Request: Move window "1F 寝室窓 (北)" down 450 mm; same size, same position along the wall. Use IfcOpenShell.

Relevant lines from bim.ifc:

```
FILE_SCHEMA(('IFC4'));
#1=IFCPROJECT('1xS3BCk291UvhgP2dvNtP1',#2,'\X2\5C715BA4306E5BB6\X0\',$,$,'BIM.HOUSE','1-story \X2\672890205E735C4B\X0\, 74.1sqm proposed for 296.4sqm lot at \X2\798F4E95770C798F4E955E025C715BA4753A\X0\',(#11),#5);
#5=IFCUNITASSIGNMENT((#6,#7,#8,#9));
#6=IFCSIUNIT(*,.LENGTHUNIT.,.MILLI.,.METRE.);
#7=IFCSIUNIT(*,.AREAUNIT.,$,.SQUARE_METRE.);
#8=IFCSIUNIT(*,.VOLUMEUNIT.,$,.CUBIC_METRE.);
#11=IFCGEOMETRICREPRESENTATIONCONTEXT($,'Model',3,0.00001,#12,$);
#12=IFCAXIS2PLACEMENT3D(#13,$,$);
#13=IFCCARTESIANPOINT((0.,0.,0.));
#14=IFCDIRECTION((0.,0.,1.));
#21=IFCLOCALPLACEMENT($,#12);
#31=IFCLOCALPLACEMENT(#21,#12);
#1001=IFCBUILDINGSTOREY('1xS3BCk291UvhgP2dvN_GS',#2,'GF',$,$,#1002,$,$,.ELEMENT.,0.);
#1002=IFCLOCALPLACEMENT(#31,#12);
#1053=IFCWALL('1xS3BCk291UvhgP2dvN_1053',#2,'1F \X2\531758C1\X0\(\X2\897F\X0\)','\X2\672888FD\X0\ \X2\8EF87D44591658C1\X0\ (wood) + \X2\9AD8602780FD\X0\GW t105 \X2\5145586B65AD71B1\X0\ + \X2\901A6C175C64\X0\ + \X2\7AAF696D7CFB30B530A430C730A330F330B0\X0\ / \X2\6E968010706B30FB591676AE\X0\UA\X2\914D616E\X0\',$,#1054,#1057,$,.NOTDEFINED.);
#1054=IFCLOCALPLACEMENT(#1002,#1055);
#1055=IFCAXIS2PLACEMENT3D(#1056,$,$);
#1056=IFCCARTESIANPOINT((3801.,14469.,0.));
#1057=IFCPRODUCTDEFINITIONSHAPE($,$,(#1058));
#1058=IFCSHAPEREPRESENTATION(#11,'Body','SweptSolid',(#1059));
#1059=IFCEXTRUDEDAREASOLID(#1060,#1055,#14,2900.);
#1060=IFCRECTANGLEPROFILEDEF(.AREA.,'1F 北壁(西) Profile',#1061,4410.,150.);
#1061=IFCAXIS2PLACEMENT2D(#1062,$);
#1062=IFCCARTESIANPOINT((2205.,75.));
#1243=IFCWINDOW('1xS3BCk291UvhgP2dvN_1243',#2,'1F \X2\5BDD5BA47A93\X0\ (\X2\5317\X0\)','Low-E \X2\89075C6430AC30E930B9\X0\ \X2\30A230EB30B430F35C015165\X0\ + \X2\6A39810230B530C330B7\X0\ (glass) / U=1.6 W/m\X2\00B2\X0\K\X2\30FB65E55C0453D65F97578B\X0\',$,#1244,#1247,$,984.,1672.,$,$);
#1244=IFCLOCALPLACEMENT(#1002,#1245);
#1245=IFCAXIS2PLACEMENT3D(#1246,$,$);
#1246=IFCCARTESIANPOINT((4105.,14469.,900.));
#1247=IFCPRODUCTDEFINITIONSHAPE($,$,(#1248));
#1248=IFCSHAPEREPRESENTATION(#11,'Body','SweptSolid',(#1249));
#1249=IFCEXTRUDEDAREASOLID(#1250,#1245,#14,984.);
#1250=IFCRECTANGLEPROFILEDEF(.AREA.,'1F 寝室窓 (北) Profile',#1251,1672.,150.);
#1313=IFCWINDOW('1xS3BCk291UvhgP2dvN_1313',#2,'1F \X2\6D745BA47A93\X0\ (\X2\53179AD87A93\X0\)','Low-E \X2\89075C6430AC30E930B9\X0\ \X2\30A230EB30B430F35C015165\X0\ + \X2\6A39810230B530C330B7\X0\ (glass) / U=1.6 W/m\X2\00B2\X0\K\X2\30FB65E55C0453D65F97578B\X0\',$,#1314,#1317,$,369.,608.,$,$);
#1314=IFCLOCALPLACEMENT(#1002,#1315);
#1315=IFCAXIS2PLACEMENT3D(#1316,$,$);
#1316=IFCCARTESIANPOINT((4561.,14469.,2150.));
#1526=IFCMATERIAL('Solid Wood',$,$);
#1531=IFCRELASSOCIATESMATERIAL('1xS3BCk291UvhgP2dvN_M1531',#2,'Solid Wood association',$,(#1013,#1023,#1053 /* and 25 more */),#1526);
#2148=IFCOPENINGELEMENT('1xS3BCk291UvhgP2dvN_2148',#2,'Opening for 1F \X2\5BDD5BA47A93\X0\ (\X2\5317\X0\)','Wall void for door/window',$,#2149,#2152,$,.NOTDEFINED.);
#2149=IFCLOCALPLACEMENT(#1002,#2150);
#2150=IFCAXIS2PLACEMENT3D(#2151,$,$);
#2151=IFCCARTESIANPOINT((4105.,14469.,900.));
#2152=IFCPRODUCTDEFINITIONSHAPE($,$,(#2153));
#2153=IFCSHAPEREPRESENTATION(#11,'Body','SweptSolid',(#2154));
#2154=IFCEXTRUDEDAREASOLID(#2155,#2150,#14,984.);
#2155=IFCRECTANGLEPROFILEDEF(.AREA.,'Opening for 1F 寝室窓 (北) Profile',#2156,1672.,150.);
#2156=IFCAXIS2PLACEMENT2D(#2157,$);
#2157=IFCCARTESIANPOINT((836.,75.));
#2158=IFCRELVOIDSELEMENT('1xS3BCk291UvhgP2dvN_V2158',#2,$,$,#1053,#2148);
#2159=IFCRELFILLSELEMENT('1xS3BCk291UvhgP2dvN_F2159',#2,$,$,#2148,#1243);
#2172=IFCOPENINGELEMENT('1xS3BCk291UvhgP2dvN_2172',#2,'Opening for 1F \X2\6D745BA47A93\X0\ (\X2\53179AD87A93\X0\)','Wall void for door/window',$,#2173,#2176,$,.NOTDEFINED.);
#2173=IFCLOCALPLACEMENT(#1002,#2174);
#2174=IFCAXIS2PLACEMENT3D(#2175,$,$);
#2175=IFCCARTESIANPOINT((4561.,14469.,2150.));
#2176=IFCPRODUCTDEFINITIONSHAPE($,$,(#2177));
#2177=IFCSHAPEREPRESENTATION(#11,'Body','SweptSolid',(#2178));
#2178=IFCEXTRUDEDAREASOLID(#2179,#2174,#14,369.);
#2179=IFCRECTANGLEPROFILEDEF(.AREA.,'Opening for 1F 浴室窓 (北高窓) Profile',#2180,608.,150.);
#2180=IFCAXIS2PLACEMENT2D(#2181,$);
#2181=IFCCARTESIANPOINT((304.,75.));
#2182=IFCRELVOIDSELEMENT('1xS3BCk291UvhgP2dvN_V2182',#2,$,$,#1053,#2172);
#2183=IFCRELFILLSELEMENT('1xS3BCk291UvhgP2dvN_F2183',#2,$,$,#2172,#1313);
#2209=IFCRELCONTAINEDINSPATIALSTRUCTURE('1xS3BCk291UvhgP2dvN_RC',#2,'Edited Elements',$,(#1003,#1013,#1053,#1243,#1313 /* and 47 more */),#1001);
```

```python
import numpy as np
import ifcopenshell
import ifcopenshell.api.geometry
import ifcopenshell.util.placement
import ifcopenshell.util.unit

model = ifcopenshell.open("bim.ifc")
unit_scale = ifcopenshell.util.unit.calculate_unit_scale(model)

window = model.by_guid("1xS3BCk291UvhgP2dvN_1243")
opening = window.FillsVoids[0].RelatingOpeningElement
dz = -0.45 / unit_scale

shift = np.array([0.0, 0.0, dz])
# The window is not placed relative to its opening, so move both.
for product in (opening, window):
    matrix = ifcopenshell.util.placement.get_local_placement(product.ObjectPlacement)
    matrix[:3, 3] += shift
    ifcopenshell.api.geometry.edit_object_placement(model, product=product, matrix=matrix, is_si=False)

print(f"moved by {dz * unit_scale:+.3f} m")

model.write("bim-out.ifc")
```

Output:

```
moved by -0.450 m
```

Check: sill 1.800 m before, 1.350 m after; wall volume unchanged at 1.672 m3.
